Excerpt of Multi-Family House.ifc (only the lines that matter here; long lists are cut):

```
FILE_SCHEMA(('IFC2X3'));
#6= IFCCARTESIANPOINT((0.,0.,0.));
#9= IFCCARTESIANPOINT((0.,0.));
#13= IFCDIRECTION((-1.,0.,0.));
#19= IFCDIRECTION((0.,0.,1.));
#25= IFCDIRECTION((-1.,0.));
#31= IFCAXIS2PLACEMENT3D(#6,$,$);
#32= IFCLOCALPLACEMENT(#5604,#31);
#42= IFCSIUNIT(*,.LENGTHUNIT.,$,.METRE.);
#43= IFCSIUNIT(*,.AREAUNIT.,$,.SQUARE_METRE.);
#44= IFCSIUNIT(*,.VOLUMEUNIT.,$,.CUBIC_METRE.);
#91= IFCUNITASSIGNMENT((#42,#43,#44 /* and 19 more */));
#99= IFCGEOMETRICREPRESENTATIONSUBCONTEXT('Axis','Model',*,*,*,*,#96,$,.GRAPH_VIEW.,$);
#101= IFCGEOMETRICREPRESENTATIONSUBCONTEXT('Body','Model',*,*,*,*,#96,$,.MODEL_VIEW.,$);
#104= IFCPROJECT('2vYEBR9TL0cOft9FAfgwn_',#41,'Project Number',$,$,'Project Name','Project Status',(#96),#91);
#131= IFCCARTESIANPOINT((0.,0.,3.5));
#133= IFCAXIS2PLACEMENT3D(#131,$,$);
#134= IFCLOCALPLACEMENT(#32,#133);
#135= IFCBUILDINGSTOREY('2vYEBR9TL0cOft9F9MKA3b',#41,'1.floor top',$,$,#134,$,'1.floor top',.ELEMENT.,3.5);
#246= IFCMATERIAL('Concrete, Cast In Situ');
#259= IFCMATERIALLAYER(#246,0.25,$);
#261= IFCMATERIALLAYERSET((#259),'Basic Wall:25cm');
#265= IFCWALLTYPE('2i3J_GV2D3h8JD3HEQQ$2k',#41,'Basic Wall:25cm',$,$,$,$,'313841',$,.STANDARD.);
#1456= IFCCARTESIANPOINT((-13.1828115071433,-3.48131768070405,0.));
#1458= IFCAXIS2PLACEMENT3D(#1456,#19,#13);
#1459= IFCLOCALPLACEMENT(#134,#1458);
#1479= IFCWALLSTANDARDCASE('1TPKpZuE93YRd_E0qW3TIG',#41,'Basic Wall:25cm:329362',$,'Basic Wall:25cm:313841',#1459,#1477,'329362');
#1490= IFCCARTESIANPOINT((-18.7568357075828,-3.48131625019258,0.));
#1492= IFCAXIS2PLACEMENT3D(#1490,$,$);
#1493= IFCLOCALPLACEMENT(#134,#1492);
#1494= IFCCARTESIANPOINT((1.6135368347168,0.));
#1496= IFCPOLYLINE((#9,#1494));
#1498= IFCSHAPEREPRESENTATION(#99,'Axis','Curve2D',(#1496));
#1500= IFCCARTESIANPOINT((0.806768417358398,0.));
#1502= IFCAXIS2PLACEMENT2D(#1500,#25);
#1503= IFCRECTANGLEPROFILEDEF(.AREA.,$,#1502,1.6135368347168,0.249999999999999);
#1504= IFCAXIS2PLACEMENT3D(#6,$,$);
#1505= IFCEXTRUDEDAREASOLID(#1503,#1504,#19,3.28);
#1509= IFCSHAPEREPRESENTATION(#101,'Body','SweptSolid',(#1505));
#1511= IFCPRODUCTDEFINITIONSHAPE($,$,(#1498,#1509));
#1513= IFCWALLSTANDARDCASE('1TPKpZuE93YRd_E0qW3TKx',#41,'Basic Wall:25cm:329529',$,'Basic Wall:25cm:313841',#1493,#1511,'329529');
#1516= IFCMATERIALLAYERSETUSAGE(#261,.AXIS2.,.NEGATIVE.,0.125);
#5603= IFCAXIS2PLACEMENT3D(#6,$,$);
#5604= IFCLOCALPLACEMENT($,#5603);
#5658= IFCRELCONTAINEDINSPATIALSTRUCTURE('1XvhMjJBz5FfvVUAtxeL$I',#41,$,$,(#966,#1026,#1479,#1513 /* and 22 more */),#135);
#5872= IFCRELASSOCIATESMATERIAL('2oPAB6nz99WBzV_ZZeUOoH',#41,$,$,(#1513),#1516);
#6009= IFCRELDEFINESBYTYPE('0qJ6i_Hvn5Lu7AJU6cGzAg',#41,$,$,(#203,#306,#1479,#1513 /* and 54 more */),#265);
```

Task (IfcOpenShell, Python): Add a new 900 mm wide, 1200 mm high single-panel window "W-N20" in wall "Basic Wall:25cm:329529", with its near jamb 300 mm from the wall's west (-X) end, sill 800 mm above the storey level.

```python
import numpy as np
import ifcopenshell
import ifcopenshell.api.feature
import ifcopenshell.api.geometry
import ifcopenshell.api.root
import ifcopenshell.api.spatial
import ifcopenshell.api.type
import ifcopenshell.geom
import ifcopenshell.util.element
import ifcopenshell.util.placement
import ifcopenshell.util.representation
import ifcopenshell.util.shape
import ifcopenshell.util.unit

model = ifcopenshell.open("Multi-Family House.ifc")
unit_scale = ifcopenshell.util.unit.calculate_unit_scale(model)
settings = ifcopenshell.geom.settings()


def volume(element):
    """Net volume in cubic metres, openings subtracted."""
    shape = ifcopenshell.geom.create_shape(settings, element)
    return ifcopenshell.util.shape.get_volume(shape.geometry)


wall = model.by_guid("1TPKpZuE93YRd_E0qW3TKx")
storey = ifcopenshell.util.element.get_container(wall, ifc_class="IfcBuildingStorey")
context = ifcopenshell.util.representation.get_context(model, "Model", "Body", "MODEL_VIEW")
before = volume(wall)

width, height, from_end, sill = 0.9, 1.2, 0.3, 0.8  # metres

# The wall runs along its own X axis, and the end named is its -X end.
wall_shape = ifcopenshell.geom.create_shape(settings, wall)
x, y, z = ifcopenshell.util.shape.get_vertices(wall_shape.geometry).T
start = x.min() + from_end
face, thickness = float(y.min()), float(y.max() - y.min())
wall_matrix = ifcopenshell.util.placement.get_local_placement(wall.ObjectPlacement)
level = ifcopenshell.util.placement.get_local_placement(storey.ObjectPlacement)[2, 3]


def in_wall(x, y):
    """Placement at x, y metres in the wall's axes, at sill height."""
    matrix = wall_matrix.copy()
    matrix[:, 3] = wall_matrix @ np.array([x / unit_scale, y / unit_scale, 0.0, 1.0])
    matrix[2, 3] = level + sill / unit_scale
    return matrix


# Opening: a box that overshoots both wall faces by 50 mm.
opening = ifcopenshell.api.root.create_entity(model, ifc_class="IfcOpeningElement")
box = ifcopenshell.api.geometry.add_wall_representation(
    model, context=context, length=width, height=height, thickness=thickness + 0.1
)
ifcopenshell.api.geometry.assign_representation(model, product=opening, representation=box)
ifcopenshell.api.geometry.edit_object_placement(model, product=opening, matrix=in_wall(start, face - 0.05), is_si=False)
ifcopenshell.api.feature.add_feature(model, feature=opening, element=wall)

window = ifcopenshell.api.root.create_entity(model, ifc_class="IfcWindow", name="W-N20")
window.OverallWidth, window.OverallHeight = width / unit_scale, height / unit_scale
body = ifcopenshell.api.geometry.add_window_representation(
    model,
    context=context,
    overall_width=window.OverallWidth,
    overall_height=window.OverallHeight,
    partition_type="SINGLE_PANEL",
)
ifcopenshell.api.geometry.assign_representation(model, product=window, representation=body)
ifcopenshell.api.spatial.assign_container(model, products=[window], relating_structure=storey)
fills = ifcopenshell.api.feature.add_filling(model, opening=opening, element=window)
fills.OwnerHistory = window.OwnerHistory  # required in IFC2X3

# IFC2X3 keeps the operation on the window style.
style = ifcopenshell.api.root.create_entity(model, ifc_class="IfcWindowStyle", name="W-N20")
style.OperationType, style.ConstructionType = "SINGLE_PANEL", "NOTDEFINED"
style.ParameterTakesPrecedence = style.Sizeable = False
ifcopenshell.api.type.assign_type(model, related_objects=[window], relating_type=style)

# Centre the window in the wall's thickness.
ifcopenshell.api.geometry.edit_object_placement(model, product=window, matrix=in_wall(start, face), is_si=False)
window_shape = ifcopenshell.geom.create_shape(settings, window)
depth = ifcopenshell.util.shape.get_vertices(window_shape.geometry)[:, 1]
offset = face + thickness / 2 - (depth.min() + depth.max()) / 2
ifcopenshell.api.geometry.edit_object_placement(model, product=window, matrix=in_wall(start, offset), is_si=False)

after = volume(wall)

print(f"wall volume {before:.3f} -> {after:.3f} m3")

model.write("Multi-Family House-out.ifc")
```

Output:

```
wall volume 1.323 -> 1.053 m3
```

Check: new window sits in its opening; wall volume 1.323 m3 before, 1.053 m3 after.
